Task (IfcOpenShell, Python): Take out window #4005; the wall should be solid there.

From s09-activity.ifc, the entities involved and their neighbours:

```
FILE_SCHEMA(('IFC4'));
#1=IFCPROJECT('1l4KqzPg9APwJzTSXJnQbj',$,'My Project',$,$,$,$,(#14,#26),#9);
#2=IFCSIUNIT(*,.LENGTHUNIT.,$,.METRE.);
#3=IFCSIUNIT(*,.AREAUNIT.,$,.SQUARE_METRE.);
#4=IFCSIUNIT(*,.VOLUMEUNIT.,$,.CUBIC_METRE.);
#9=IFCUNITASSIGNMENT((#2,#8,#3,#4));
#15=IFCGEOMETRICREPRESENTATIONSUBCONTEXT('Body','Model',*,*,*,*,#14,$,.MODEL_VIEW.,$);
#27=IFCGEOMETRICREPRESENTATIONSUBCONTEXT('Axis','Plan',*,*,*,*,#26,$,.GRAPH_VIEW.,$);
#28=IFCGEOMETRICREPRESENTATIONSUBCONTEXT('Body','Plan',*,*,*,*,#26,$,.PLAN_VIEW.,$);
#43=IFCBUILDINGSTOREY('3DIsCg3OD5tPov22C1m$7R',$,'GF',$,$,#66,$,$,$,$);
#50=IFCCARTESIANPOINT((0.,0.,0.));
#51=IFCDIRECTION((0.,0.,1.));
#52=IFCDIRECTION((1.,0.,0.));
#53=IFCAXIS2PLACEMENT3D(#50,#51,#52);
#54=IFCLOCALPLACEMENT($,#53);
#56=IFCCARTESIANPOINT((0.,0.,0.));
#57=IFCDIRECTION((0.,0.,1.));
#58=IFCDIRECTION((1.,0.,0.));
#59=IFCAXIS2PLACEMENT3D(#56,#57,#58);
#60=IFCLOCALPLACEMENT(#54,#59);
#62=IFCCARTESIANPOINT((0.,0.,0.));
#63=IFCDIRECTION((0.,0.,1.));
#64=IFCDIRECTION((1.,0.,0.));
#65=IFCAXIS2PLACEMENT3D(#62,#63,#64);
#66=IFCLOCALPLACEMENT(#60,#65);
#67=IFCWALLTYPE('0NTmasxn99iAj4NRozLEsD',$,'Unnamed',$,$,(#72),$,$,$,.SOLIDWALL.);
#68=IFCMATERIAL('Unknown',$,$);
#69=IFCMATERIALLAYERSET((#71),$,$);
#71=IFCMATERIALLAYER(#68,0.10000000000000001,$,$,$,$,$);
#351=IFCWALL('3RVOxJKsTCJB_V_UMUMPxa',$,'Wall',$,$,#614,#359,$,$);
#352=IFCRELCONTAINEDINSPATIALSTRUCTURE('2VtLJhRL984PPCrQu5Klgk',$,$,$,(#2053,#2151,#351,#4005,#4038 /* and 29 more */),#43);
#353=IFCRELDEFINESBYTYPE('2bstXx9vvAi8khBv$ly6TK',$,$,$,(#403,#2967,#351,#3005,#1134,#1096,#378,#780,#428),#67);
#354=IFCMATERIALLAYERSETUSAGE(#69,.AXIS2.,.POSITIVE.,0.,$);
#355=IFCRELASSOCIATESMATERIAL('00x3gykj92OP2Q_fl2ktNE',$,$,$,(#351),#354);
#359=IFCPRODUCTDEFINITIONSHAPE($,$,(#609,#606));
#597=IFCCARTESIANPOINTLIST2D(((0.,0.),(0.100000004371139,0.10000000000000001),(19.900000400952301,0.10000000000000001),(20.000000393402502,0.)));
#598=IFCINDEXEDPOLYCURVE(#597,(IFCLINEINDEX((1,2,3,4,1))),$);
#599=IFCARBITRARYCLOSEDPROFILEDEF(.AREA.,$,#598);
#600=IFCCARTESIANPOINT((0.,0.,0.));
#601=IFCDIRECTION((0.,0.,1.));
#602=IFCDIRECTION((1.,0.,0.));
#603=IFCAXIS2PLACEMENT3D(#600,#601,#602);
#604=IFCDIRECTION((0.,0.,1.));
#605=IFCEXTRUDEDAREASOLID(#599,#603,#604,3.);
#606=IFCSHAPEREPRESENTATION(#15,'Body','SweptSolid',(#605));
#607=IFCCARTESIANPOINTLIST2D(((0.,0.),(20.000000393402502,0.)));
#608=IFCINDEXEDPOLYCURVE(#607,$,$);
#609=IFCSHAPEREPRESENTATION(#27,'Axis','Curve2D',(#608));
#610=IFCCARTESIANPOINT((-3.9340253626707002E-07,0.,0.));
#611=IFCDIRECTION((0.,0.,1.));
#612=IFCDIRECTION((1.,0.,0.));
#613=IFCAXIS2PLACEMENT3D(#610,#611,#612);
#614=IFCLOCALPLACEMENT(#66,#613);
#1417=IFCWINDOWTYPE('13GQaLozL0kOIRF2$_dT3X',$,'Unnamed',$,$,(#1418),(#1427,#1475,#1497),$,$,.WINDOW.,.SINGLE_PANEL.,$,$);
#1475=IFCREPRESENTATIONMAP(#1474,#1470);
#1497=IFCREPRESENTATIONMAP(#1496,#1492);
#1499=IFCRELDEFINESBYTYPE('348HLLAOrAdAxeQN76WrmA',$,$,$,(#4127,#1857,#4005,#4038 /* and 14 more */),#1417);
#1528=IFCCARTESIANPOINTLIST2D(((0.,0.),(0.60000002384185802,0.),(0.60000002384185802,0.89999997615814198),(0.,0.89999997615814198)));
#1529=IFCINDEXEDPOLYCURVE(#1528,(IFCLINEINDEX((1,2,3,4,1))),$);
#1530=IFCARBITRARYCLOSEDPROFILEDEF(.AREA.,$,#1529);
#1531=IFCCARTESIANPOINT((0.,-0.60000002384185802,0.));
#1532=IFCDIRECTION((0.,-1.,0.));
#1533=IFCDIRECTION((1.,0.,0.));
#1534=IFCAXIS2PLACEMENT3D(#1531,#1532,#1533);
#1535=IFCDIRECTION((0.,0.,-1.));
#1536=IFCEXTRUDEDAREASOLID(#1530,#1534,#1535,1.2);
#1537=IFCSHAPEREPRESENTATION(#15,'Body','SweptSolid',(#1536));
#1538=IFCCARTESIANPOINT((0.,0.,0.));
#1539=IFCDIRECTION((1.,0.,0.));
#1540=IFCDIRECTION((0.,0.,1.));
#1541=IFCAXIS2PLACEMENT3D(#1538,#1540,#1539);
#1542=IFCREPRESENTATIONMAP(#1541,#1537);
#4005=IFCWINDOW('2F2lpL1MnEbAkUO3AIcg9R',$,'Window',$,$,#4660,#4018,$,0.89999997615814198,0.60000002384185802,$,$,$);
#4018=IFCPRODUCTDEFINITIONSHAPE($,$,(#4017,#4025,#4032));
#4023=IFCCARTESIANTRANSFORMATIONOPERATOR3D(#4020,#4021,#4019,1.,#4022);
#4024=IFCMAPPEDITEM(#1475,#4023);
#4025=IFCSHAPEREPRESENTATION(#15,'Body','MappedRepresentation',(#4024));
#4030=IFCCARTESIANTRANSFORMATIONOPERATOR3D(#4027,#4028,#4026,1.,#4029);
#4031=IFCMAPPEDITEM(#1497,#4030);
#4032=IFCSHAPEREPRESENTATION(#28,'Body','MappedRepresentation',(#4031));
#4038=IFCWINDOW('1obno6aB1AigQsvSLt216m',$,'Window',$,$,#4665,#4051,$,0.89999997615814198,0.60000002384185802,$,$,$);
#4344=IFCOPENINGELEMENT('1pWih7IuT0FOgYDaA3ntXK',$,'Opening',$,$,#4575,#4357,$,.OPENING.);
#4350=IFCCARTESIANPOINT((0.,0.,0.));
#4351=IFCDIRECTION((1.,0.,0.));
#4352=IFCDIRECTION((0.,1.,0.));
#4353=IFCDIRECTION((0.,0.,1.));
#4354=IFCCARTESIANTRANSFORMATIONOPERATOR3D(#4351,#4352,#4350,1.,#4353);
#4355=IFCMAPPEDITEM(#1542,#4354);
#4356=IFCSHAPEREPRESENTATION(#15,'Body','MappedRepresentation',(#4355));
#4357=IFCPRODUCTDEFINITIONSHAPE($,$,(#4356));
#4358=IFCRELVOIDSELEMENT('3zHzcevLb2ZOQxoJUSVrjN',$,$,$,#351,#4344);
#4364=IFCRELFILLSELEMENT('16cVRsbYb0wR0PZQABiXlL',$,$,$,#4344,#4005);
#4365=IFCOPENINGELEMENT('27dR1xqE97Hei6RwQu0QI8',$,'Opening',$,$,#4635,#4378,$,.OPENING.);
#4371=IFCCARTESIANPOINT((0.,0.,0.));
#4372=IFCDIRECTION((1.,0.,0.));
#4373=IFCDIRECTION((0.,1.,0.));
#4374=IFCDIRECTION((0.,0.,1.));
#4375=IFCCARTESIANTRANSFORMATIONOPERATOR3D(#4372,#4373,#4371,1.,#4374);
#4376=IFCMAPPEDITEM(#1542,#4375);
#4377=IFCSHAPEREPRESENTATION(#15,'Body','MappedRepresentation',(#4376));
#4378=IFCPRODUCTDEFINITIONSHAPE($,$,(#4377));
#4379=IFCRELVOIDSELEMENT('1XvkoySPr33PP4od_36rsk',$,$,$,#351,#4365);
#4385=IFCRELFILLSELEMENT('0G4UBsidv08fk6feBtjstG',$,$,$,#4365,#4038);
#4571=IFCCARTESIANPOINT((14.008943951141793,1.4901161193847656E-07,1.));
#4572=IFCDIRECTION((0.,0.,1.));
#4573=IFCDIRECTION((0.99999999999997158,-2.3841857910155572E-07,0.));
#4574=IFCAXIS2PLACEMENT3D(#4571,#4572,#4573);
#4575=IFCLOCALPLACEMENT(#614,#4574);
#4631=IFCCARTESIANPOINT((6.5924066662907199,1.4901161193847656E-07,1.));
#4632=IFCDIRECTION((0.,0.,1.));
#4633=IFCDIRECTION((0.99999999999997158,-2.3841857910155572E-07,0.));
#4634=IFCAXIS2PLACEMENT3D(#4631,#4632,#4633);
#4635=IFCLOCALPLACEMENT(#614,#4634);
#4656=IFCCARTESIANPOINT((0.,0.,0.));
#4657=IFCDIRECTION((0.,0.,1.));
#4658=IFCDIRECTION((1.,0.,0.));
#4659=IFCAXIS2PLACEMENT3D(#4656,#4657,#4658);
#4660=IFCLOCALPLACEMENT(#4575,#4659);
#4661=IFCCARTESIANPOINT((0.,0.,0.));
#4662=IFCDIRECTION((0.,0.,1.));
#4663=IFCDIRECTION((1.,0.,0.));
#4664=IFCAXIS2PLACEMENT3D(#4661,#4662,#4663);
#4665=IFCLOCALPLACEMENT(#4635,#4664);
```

```python
import ifcopenshell
import ifcopenshell.api.feature
import ifcopenshell.api.root
import ifcopenshell.geom
import ifcopenshell.util.shape

model = ifcopenshell.open("s09-activity.ifc")
settings = ifcopenshell.geom.settings()


def volume(element):
    """Net volume in cubic metres, openings subtracted."""
    shape = ifcopenshell.geom.create_shape(settings, element)
    return ifcopenshell.util.shape.get_volume(shape.geometry)


window = model.by_id(4005)
opening = window.FillsVoids[0].RelatingOpeningElement
wall = opening.VoidsElements[0].RelatingBuildingElement
before = volume(wall)

ifcopenshell.api.root.remove_product(model, product=window)
ifcopenshell.api.feature.remove_feature(model, feature=opening)

after = volume(wall)

print(f"wall volume {before:.3f} -> {after:.3f} m3")

model.write("s09-activity_updated.ifc")
```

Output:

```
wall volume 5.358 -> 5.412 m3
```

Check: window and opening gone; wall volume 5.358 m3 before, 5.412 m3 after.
